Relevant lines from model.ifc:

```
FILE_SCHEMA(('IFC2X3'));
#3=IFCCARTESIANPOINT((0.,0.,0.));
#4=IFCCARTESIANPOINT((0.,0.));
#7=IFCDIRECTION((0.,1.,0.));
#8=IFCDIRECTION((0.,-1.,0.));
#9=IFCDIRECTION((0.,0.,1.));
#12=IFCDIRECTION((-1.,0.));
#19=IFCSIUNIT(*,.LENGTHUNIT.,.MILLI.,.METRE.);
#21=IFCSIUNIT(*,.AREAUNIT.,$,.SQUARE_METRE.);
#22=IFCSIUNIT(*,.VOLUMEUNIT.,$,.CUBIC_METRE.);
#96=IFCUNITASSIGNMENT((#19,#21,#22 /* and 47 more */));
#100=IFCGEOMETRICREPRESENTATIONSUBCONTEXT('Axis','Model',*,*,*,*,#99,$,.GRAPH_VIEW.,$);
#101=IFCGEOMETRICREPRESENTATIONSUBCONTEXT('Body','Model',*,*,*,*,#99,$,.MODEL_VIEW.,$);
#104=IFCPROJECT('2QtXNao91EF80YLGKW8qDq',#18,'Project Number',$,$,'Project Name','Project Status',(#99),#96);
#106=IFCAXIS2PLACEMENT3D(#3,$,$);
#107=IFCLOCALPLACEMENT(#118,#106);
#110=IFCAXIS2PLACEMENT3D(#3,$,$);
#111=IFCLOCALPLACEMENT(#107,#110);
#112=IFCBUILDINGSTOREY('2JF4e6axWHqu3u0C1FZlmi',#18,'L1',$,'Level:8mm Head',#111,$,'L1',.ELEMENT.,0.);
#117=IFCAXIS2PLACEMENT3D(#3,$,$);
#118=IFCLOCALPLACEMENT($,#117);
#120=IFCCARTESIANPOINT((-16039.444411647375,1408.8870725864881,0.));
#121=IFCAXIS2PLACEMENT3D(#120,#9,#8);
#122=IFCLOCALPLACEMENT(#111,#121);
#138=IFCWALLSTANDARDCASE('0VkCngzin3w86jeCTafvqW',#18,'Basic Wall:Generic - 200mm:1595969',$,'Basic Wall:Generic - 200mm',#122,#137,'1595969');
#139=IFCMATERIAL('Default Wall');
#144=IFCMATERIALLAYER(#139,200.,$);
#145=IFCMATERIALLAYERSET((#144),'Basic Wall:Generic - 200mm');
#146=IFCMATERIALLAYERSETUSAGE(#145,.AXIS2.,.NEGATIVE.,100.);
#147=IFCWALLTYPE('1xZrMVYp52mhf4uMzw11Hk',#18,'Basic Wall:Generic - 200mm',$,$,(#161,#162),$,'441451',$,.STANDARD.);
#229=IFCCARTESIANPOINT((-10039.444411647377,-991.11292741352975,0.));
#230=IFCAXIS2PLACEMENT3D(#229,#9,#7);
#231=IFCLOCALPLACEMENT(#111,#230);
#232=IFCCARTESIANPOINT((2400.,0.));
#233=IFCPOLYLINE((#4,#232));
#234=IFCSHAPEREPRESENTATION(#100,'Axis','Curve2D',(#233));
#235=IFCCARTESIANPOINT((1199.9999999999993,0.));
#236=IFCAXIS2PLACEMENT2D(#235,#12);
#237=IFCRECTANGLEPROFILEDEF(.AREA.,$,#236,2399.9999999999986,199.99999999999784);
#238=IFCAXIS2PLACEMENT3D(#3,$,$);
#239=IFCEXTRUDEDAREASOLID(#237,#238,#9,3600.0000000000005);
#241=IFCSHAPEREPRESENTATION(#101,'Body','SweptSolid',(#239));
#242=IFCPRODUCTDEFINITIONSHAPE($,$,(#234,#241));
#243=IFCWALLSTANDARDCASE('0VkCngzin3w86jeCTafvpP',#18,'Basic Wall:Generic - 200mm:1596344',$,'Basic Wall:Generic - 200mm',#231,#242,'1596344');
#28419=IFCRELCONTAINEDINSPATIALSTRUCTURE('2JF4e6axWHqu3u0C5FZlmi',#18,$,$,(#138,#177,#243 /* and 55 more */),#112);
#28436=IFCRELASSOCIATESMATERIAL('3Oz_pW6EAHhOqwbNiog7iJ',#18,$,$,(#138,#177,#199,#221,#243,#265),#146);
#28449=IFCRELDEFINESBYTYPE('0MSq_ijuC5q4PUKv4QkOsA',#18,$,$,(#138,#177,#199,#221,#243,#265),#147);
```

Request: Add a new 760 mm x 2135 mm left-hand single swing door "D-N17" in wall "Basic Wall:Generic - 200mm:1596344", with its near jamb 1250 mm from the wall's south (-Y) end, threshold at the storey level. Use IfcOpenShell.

```python
import numpy as np
import ifcopenshell
import ifcopenshell.api.feature
import ifcopenshell.api.geometry
import ifcopenshell.api.root
import ifcopenshell.api.spatial
import ifcopenshell.api.type
import ifcopenshell.geom
import ifcopenshell.util.element
import ifcopenshell.util.placement
import ifcopenshell.util.representation
import ifcopenshell.util.shape
import ifcopenshell.util.unit

model = ifcopenshell.open("model.ifc")
unit_scale = ifcopenshell.util.unit.calculate_unit_scale(model)
settings = ifcopenshell.geom.settings()


def volume(element):
    """Net volume in cubic metres, openings subtracted."""
    shape = ifcopenshell.geom.create_shape(settings, element)
    return ifcopenshell.util.shape.get_volume(shape.geometry)


wall = model.by_id(243)
storey = ifcopenshell.util.element.get_container(wall, ifc_class="IfcBuildingStorey")
context = ifcopenshell.util.representation.get_context(model, "Model", "Body", "MODEL_VIEW")
before = volume(wall)

width, height, from_end, sill = 0.76, 2.135, 1.25, 0.0  # metres

# The wall runs along its own X axis, and the end named is its -X end.
wall_shape = ifcopenshell.geom.create_shape(settings, wall)
x, y, z = ifcopenshell.util.shape.get_vertices(wall_shape.geometry).T
start = x.min() + from_end
face, thickness = float(y.min()), float(y.max() - y.min())
wall_matrix = ifcopenshell.util.placement.get_local_placement(wall.ObjectPlacement)
level = ifcopenshell.util.placement.get_local_placement(storey.ObjectPlacement)[2, 3]


def in_wall(x, y):
    """Placement at x, y metres in the wall's axes, at sill height."""
    matrix = wall_matrix.copy()
    matrix[:, 3] = wall_matrix @ np.array([x / unit_scale, y / unit_scale, 0.0, 1.0])
    matrix[2, 3] = level + sill / unit_scale
    return matrix


# Opening: a box that overshoots both wall faces by 50 mm.
opening = ifcopenshell.api.root.create_entity(model, ifc_class="IfcOpeningElement")
box = ifcopenshell.api.geometry.add_wall_representation(
    model, context=context, length=width, height=height, thickness=thickness + 0.1
)
ifcopenshell.api.geometry.assign_representation(model, product=opening, representation=box)
ifcopenshell.api.geometry.edit_object_placement(model, product=opening, matrix=in_wall(start, face - 0.05), is_si=False)
ifcopenshell.api.feature.add_feature(model, feature=opening, element=wall)

door = ifcopenshell.api.root.create_entity(model, ifc_class="IfcDoor", name="D-N17")
door.OverallWidth, door.OverallHeight = width / unit_scale, height / unit_scale
body = ifcopenshell.api.geometry.add_door_representation(
    model,
    context=context,
    overall_width=door.OverallWidth,
    overall_height=door.OverallHeight,
    operation_type="SINGLE_SWING_LEFT",
    lining_properties={"LiningDepth": thickness / unit_scale, "ThresholdDepth": thickness / unit_scale},
)
ifcopenshell.api.geometry.assign_representation(model, product=door, representation=body)
ifcopenshell.api.spatial.assign_container(model, products=[door], relating_structure=storey)
fills = ifcopenshell.api.feature.add_filling(model, opening=opening, element=door)
fills.OwnerHistory = door.OwnerHistory  # required in IFC2X3

# IFC2X3 keeps the operation on the door style.
style = ifcopenshell.api.root.create_entity(model, ifc_class="IfcDoorStyle", name="D-N17")
style.OperationType, style.ConstructionType = "SINGLE_SWING_LEFT", "NOTDEFINED"
style.ParameterTakesPrecedence = style.Sizeable = False
ifcopenshell.api.type.assign_type(model, related_objects=[door], relating_type=style)

# The lining spans the wall, so the door starts at the wall face.
ifcopenshell.api.geometry.edit_object_placement(model, product=door, matrix=in_wall(start, face), is_si=False)

after = volume(wall)

print(f"wall volume {before:.3f} -> {after:.3f} m3")

model.write("model_edited.ifc")
```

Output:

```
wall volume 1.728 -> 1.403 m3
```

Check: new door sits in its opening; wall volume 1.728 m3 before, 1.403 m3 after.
